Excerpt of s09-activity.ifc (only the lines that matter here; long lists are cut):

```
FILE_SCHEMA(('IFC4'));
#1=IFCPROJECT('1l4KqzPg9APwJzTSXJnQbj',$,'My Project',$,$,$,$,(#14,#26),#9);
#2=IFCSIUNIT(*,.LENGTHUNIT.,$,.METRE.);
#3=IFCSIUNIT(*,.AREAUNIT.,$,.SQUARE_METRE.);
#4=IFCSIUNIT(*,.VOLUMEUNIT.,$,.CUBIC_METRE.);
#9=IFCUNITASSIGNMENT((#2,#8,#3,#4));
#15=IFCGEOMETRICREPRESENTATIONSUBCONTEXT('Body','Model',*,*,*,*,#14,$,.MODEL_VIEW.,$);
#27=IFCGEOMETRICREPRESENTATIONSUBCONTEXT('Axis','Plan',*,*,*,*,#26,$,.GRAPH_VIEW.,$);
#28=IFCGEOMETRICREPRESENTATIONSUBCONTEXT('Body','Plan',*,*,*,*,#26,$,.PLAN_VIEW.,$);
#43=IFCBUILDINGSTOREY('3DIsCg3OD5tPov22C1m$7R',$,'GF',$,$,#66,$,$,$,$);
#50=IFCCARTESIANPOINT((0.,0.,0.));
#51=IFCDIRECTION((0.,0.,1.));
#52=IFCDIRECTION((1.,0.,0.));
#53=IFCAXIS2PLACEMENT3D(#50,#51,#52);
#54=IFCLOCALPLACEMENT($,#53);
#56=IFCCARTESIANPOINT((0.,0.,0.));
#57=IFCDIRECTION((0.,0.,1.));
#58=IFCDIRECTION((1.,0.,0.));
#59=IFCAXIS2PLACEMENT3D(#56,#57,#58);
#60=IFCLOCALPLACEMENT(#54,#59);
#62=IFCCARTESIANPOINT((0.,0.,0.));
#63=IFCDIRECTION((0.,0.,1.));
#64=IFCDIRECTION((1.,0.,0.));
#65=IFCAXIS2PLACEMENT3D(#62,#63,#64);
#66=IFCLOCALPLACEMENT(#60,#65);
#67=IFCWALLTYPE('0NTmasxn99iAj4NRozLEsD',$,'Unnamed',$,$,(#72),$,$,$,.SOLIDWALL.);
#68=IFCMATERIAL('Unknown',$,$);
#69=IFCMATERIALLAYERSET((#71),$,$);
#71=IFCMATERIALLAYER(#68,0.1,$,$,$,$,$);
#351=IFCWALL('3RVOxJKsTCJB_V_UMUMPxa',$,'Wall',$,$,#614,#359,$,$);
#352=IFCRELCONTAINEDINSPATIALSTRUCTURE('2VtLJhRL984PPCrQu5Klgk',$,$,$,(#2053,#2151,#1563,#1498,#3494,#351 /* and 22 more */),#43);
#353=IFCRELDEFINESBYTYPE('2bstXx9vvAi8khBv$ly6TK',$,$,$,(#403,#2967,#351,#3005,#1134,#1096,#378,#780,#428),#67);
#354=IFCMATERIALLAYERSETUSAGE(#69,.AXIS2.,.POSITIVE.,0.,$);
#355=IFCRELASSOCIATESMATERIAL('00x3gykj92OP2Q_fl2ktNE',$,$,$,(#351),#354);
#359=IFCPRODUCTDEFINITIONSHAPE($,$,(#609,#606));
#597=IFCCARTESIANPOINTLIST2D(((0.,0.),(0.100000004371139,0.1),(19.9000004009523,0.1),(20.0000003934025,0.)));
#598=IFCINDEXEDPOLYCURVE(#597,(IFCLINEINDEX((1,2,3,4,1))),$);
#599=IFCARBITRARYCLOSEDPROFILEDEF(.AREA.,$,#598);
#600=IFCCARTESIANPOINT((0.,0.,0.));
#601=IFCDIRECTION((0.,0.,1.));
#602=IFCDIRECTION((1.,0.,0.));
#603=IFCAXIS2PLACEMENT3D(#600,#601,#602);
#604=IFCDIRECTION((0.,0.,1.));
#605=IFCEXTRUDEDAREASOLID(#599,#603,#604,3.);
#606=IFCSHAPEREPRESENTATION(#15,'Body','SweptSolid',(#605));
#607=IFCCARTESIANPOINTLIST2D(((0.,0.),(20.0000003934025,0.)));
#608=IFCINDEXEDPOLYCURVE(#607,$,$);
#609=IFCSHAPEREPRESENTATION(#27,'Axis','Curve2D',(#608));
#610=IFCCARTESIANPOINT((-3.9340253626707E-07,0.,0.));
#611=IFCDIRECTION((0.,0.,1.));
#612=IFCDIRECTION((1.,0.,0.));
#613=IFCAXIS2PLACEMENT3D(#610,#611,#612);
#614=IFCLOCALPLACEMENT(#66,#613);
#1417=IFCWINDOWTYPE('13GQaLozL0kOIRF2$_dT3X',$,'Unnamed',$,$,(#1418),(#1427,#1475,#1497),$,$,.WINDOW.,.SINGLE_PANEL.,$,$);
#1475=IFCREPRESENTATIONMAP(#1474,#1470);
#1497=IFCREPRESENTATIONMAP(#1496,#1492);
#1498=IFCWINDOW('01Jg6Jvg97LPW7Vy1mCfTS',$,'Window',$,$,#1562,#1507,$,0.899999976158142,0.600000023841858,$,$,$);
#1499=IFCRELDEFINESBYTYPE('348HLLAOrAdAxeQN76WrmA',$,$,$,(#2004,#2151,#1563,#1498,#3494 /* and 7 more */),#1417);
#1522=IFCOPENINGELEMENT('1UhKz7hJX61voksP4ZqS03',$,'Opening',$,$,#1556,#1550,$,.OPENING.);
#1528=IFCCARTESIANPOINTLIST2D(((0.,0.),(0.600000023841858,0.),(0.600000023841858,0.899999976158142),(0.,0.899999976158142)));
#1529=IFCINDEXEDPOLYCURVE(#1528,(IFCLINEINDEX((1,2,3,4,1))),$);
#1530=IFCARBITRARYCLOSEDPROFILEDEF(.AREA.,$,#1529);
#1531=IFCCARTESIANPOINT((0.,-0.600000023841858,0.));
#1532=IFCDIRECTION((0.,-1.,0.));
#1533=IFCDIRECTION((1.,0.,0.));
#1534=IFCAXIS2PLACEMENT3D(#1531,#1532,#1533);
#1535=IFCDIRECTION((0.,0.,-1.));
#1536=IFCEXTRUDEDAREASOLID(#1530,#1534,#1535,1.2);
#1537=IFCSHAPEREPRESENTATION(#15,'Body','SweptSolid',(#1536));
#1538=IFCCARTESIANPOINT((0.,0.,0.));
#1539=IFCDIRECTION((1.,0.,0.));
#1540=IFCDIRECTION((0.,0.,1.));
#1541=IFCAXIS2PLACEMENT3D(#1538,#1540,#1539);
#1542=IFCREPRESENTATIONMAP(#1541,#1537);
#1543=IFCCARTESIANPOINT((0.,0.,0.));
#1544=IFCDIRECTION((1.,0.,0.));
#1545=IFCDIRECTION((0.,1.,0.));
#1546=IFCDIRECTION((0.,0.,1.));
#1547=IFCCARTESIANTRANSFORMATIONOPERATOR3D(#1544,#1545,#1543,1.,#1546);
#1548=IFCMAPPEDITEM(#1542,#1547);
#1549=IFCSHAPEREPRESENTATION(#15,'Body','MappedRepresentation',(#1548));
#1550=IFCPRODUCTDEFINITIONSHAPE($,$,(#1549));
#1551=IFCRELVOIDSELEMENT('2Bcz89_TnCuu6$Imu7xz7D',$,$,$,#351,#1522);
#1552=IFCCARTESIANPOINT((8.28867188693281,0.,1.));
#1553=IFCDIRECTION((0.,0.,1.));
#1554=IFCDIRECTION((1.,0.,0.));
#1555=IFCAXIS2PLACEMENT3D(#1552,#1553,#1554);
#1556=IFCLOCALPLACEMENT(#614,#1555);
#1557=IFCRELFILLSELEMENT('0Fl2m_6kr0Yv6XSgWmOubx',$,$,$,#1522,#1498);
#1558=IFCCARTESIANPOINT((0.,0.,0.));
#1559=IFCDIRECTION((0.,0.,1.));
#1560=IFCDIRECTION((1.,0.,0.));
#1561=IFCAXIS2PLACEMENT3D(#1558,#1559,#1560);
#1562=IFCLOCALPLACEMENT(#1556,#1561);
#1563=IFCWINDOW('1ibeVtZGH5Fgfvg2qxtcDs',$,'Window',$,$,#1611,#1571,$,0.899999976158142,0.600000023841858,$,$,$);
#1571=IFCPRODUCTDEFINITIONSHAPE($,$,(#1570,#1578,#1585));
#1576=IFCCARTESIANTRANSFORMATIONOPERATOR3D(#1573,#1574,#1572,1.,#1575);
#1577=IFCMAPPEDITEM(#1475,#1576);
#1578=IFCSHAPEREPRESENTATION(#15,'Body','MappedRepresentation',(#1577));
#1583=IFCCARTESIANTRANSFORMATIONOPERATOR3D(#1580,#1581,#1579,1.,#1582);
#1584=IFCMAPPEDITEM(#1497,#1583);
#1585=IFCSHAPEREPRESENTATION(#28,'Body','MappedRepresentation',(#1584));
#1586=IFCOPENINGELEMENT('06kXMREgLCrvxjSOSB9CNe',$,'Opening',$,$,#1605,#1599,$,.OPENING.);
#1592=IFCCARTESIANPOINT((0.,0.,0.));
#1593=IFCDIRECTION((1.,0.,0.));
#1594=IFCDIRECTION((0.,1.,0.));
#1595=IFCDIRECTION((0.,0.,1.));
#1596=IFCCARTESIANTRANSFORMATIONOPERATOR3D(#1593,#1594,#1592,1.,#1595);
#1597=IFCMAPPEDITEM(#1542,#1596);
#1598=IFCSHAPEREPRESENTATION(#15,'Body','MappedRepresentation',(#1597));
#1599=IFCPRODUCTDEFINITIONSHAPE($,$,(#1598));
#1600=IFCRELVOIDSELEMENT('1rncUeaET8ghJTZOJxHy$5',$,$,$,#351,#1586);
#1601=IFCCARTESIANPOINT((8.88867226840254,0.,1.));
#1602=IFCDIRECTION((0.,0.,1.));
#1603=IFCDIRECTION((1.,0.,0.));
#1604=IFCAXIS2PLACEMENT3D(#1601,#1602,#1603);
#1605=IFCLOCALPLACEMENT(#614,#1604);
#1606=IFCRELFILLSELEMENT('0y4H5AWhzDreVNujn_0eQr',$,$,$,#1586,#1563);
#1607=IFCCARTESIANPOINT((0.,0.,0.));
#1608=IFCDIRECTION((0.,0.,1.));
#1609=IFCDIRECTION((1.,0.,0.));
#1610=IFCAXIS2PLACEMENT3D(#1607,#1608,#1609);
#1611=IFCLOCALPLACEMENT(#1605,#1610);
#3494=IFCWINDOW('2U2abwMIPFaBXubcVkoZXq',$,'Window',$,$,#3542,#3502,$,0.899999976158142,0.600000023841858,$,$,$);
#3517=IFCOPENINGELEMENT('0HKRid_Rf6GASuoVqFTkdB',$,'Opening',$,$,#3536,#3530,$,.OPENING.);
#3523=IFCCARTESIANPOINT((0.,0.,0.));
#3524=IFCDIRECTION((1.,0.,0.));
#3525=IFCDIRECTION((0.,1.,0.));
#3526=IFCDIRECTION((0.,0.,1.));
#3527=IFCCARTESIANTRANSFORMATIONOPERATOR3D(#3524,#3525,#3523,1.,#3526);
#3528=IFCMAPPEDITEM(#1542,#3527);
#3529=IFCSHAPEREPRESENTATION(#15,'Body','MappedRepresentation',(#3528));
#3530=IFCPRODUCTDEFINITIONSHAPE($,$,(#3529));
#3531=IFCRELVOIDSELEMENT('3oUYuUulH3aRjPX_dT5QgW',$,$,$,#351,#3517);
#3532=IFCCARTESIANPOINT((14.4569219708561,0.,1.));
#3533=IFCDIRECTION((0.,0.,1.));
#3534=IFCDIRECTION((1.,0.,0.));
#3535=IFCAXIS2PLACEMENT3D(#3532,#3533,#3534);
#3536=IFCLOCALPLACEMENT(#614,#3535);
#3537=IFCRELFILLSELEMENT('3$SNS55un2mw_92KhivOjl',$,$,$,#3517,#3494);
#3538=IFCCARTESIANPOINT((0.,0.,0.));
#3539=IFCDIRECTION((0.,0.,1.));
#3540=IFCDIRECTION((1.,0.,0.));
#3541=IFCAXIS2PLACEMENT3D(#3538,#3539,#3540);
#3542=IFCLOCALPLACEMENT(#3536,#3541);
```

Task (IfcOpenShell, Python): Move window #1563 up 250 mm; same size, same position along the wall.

```python
import numpy as np
import ifcopenshell
import ifcopenshell.api.geometry
import ifcopenshell.util.placement
import ifcopenshell.util.unit

model = ifcopenshell.open("s09-activity.ifc")
unit_scale = ifcopenshell.util.unit.calculate_unit_scale(model)

window = model.by_guid("1ibeVtZGH5Fgfvg2qxtcDs")
opening = window.FillsVoids[0].RelatingOpeningElement
dz = 0.25 / unit_scale

shift = np.array([0.0, 0.0, dz])
# The window is placed relative to its opening, so it follows when the opening moves.
matrix = ifcopenshell.util.placement.get_local_placement(opening.ObjectPlacement)
matrix[:3, 3] += shift
ifcopenshell.api.geometry.edit_object_placement(
    model, product=opening, matrix=matrix, is_si=False, should_transform_children=True
)

print(f"moved by {dz * unit_scale:+.3f} m")

model.write("s09-activity-out.ifc")
```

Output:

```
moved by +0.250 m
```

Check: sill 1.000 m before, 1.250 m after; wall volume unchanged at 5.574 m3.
